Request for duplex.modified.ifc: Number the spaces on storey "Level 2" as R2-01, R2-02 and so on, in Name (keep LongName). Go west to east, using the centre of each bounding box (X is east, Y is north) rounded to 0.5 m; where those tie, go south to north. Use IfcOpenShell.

First a look at what the model holds.

```python
import ifcopenshell
import ifcopenshell.util.element
import ifcopenshell.util.placement

model = ifcopenshell.open("duplex.modified.ifc")
print(model.schema)
storey = next(s for s in model.by_type("IfcBuildingStorey") if s.Name == "Level 2")
spaces = [e for e in ifcopenshell.util.element.get_decomposition(storey) if e.is_a("IfcSpace")]
for e in sorted(spaces, key=lambda e: e.id()):
    origin = ifcopenshell.util.placement.get_local_placement(e.ObjectPlacement)[:3, 3]
    print(e.id(), e.Name, e.LongName, origin.round(2) + 0.0, sep=" | ")
```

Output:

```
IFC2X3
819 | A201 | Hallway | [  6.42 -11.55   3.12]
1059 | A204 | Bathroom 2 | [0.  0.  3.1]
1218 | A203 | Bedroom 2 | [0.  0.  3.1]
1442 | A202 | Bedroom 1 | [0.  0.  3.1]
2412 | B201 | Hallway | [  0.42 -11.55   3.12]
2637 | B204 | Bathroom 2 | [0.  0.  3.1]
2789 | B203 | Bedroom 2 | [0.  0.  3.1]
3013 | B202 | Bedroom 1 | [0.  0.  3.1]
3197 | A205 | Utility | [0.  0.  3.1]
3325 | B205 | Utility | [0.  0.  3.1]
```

```python
import ifcopenshell
import ifcopenshell.geom
import ifcopenshell.util.element
import ifcopenshell.util.shape

model = ifcopenshell.open("duplex.modified.ifc")
settings = ifcopenshell.geom.settings()
settings.set("use-world-coords", True)


def centre(element):
    shape = ifcopenshell.geom.create_shape(settings, element)
    return ifcopenshell.util.shape.get_bbox_centroid(shape.geometry)


storey = next(s for s in model.by_type("IfcBuildingStorey") if s.Name == "Level 2")
spaces = [e for e in ifcopenshell.util.element.get_decomposition(storey) if e.is_a("IfcSpace")]

# Insertion points can sit at a corner or the storey origin, so sort by the geometry (in metres).
centres = {e: centre(e) for e in spaces}
spaces.sort(key=lambda e: (round(centres[e][0] / 0.5), centres[e][1]))

for i, e in enumerate(spaces, start=1):
    number = f"R2-{i:02d}"
    e.Name = number
    print(e.id(), number)

model.write("duplex.modified_updated.ifc")
```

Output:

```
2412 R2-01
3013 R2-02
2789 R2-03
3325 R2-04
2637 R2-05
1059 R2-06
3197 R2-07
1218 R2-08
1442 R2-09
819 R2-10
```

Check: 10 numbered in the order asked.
